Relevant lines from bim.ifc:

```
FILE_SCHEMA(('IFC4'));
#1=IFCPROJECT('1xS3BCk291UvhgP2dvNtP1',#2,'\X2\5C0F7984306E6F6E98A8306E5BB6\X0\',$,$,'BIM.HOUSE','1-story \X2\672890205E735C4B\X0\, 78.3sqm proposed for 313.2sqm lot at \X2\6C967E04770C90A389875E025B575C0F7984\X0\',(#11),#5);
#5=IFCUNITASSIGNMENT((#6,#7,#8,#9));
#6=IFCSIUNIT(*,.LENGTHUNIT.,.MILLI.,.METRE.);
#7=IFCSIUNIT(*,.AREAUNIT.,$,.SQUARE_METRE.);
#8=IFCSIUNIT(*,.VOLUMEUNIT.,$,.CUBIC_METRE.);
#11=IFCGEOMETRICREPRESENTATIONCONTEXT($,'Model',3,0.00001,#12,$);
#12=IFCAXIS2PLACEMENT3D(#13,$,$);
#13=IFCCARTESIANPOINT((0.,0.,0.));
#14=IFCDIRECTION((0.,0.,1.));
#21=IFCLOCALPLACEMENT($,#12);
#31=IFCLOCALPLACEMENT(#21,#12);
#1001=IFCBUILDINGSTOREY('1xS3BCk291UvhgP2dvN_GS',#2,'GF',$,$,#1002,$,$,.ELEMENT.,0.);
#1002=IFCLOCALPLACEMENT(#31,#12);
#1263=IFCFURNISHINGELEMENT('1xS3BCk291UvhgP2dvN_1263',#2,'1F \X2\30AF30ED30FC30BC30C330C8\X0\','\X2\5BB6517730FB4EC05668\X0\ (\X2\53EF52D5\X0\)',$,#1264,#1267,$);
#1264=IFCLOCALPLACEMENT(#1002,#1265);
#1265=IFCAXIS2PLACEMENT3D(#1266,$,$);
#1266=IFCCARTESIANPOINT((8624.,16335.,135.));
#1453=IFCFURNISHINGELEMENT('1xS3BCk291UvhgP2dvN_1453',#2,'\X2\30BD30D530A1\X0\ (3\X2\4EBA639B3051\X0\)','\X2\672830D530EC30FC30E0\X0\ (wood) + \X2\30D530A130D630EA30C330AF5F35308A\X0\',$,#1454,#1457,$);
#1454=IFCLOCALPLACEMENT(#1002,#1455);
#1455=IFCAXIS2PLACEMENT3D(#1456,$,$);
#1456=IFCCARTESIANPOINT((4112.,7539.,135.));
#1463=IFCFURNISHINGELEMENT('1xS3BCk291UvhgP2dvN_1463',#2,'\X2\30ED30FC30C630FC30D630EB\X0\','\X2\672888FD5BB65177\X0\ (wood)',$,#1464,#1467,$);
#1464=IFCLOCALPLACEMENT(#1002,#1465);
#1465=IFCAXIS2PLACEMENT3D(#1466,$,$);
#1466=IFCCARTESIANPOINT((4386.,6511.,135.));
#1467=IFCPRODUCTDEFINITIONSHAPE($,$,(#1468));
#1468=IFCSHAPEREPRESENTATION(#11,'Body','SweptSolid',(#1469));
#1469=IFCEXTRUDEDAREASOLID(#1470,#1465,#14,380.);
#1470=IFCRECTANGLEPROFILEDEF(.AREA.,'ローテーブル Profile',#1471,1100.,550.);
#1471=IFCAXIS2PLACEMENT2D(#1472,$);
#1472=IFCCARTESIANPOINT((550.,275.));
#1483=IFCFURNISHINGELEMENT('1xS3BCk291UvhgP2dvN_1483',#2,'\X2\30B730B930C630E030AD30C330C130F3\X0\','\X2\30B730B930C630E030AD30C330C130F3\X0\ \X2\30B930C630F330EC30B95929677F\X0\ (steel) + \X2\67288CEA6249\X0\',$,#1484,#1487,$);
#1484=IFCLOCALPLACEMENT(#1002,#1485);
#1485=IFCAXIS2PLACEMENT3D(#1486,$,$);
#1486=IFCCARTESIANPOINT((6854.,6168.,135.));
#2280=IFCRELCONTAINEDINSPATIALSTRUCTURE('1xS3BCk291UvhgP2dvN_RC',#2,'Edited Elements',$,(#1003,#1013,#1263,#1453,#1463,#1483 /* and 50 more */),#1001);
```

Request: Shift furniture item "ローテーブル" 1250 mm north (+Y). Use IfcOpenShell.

```python
import ifcopenshell
import ifcopenshell.api.geometry
import ifcopenshell.util.placement

model = ifcopenshell.open("bim.ifc")

item = model.by_guid("1xS3BCk291UvhgP2dvN_1463")
matrix = ifcopenshell.util.placement.get_local_placement(item.ObjectPlacement)
matrix[1, 3] += 1250.0
ifcopenshell.api.geometry.edit_object_placement(model, product=item, matrix=matrix, is_si=False)

print(ifcopenshell.util.placement.get_local_placement(item.ObjectPlacement).round(3) + 0.0)

model.write("bim_updated.ifc")
```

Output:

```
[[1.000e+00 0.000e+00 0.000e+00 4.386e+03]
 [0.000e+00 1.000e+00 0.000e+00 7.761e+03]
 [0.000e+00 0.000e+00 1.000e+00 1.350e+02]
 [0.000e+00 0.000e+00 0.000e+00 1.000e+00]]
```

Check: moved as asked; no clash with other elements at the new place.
